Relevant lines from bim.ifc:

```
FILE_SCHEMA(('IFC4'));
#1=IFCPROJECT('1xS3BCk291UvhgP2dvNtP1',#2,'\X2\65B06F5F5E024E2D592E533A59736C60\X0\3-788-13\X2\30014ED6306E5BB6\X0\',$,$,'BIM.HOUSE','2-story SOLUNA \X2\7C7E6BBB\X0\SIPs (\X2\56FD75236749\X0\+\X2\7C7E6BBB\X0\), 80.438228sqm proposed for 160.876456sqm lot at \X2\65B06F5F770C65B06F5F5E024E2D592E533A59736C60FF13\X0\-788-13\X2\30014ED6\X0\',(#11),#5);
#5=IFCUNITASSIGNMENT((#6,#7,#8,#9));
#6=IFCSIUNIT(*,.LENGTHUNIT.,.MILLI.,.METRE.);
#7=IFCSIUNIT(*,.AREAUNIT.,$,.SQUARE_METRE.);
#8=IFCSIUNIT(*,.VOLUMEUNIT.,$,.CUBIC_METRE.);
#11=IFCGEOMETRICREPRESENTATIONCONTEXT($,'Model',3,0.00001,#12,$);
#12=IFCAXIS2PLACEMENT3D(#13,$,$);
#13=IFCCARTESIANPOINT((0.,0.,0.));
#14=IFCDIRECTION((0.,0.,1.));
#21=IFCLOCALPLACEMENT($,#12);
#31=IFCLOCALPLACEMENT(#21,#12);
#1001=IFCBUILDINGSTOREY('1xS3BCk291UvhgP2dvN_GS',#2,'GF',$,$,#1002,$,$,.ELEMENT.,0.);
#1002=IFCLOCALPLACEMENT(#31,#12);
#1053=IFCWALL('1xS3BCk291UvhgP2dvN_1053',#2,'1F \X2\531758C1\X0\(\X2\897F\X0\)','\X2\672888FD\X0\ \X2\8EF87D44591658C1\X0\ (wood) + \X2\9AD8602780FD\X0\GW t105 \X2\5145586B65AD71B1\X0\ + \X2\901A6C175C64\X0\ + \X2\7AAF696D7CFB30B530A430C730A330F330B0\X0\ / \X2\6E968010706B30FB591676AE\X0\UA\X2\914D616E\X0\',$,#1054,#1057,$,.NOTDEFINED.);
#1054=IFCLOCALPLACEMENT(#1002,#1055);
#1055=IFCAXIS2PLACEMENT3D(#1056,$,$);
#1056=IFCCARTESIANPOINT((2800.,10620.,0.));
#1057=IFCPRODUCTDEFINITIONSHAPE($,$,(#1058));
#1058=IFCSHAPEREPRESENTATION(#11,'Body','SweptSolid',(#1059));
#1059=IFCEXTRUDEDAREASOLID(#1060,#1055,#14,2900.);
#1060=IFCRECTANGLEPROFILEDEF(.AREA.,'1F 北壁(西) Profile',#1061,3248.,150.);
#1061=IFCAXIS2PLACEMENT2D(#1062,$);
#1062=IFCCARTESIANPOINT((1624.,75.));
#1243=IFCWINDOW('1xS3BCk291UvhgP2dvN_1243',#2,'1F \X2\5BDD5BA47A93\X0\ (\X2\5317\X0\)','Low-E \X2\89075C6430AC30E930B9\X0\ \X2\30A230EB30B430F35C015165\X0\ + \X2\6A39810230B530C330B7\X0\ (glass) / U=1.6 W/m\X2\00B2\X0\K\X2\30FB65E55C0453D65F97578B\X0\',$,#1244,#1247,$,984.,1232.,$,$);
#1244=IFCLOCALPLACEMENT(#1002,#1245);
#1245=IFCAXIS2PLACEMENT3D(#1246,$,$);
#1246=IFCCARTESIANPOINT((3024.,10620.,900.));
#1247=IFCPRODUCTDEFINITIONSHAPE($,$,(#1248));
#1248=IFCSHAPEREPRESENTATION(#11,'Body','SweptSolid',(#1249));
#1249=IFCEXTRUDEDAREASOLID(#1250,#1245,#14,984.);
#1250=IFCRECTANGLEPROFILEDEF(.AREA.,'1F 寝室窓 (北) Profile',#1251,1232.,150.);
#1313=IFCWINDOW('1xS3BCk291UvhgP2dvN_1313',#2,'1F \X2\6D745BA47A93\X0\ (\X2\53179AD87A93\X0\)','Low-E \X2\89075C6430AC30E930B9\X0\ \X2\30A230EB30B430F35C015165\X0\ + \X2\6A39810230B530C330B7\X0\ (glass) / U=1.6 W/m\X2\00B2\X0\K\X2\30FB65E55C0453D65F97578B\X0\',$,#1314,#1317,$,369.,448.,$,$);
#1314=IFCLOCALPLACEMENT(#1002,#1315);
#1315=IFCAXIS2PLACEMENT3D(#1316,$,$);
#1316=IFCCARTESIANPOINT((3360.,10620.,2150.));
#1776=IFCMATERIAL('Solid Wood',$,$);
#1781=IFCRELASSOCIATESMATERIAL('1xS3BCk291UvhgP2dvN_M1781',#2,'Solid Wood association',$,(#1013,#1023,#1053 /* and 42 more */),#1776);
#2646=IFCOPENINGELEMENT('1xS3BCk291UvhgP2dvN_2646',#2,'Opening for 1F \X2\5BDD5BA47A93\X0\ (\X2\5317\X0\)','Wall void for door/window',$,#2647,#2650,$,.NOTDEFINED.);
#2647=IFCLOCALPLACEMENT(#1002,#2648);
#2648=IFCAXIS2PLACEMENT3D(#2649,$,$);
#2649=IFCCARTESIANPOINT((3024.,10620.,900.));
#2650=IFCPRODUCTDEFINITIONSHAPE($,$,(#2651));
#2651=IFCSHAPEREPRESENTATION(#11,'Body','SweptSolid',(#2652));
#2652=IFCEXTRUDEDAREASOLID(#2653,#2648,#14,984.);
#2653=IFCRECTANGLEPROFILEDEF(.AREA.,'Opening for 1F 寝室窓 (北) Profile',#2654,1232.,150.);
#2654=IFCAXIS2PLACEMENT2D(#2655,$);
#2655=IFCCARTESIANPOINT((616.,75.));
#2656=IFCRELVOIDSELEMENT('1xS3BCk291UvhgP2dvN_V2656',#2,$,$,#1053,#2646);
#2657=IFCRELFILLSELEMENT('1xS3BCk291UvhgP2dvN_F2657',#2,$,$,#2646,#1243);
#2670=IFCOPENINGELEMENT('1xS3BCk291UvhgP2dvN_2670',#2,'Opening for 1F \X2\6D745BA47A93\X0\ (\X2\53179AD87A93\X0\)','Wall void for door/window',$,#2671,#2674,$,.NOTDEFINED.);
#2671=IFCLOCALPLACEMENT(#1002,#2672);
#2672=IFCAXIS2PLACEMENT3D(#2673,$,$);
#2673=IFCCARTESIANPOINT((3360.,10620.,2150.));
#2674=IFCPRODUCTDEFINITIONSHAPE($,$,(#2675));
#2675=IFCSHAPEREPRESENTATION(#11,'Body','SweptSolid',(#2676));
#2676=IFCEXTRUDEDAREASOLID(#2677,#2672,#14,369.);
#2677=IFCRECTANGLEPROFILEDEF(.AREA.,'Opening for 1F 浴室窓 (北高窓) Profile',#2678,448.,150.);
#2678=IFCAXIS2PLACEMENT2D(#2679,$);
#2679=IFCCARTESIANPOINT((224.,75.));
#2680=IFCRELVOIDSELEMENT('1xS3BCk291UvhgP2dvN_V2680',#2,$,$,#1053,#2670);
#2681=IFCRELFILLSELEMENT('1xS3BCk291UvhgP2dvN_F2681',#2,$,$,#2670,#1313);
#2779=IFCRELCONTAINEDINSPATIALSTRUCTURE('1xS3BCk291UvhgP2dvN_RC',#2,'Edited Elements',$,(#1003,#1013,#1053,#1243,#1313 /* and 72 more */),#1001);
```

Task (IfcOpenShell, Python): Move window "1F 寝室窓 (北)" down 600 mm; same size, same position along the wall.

```python
import numpy as np
import ifcopenshell
import ifcopenshell.api.geometry
import ifcopenshell.util.placement
import ifcopenshell.util.unit

model = ifcopenshell.open("bim.ifc")
unit_scale = ifcopenshell.util.unit.calculate_unit_scale(model)

window = model.by_guid("1xS3BCk291UvhgP2dvN_1243")
opening = window.FillsVoids[0].RelatingOpeningElement
dz = -0.6 / unit_scale

shift = np.array([0.0, 0.0, dz])
# The window is not placed relative to its opening, so move both.
for product in (opening, window):
    matrix = ifcopenshell.util.placement.get_local_placement(product.ObjectPlacement)
    matrix[:3, 3] += shift
    ifcopenshell.api.geometry.edit_object_placement(model, product=product, matrix=matrix, is_si=False)

print(f"moved by {dz * unit_scale:+.3f} m")

model.write("bim_edited.ifc")
```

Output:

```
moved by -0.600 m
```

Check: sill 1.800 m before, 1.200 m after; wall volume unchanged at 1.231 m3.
